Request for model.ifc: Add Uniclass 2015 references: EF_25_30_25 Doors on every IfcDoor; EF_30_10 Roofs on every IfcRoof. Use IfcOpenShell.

First a look at what the model holds.

```python
import ifcopenshell

model = ifcopenshell.open("model.ifc")
print(model.schema)
print("classifications:", [c.Name for c in model.by_type("IfcClassification")])
for ifc_class in ("IfcDoor", "IfcRoof", "IfcStair", "IfcWall", "IfcWindow"):
    print(ifc_class, len(model.by_type(ifc_class)))
```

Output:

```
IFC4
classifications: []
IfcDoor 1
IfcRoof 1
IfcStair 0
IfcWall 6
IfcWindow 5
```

```python
import ifcopenshell
import ifcopenshell.api.classification

model = ifcopenshell.open("model.ifc")

system = ifcopenshell.api.classification.add_classification(model, classification="Uniclass 2015")

codes = {
    "IfcDoor": ("EF_25_30_25", "Doors"),
    "IfcRoof": ("EF_30_10", "Roofs"),
}
for ifc_class, (code, name) in codes.items():
    products = model.by_type(ifc_class)
    ifcopenshell.api.classification.add_reference(
        model, products=products, classification=system, identification=code, name=name
    )
    print(code, len(products))

model.write("model-out.ifc")
```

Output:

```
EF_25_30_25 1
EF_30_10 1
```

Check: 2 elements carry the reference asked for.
